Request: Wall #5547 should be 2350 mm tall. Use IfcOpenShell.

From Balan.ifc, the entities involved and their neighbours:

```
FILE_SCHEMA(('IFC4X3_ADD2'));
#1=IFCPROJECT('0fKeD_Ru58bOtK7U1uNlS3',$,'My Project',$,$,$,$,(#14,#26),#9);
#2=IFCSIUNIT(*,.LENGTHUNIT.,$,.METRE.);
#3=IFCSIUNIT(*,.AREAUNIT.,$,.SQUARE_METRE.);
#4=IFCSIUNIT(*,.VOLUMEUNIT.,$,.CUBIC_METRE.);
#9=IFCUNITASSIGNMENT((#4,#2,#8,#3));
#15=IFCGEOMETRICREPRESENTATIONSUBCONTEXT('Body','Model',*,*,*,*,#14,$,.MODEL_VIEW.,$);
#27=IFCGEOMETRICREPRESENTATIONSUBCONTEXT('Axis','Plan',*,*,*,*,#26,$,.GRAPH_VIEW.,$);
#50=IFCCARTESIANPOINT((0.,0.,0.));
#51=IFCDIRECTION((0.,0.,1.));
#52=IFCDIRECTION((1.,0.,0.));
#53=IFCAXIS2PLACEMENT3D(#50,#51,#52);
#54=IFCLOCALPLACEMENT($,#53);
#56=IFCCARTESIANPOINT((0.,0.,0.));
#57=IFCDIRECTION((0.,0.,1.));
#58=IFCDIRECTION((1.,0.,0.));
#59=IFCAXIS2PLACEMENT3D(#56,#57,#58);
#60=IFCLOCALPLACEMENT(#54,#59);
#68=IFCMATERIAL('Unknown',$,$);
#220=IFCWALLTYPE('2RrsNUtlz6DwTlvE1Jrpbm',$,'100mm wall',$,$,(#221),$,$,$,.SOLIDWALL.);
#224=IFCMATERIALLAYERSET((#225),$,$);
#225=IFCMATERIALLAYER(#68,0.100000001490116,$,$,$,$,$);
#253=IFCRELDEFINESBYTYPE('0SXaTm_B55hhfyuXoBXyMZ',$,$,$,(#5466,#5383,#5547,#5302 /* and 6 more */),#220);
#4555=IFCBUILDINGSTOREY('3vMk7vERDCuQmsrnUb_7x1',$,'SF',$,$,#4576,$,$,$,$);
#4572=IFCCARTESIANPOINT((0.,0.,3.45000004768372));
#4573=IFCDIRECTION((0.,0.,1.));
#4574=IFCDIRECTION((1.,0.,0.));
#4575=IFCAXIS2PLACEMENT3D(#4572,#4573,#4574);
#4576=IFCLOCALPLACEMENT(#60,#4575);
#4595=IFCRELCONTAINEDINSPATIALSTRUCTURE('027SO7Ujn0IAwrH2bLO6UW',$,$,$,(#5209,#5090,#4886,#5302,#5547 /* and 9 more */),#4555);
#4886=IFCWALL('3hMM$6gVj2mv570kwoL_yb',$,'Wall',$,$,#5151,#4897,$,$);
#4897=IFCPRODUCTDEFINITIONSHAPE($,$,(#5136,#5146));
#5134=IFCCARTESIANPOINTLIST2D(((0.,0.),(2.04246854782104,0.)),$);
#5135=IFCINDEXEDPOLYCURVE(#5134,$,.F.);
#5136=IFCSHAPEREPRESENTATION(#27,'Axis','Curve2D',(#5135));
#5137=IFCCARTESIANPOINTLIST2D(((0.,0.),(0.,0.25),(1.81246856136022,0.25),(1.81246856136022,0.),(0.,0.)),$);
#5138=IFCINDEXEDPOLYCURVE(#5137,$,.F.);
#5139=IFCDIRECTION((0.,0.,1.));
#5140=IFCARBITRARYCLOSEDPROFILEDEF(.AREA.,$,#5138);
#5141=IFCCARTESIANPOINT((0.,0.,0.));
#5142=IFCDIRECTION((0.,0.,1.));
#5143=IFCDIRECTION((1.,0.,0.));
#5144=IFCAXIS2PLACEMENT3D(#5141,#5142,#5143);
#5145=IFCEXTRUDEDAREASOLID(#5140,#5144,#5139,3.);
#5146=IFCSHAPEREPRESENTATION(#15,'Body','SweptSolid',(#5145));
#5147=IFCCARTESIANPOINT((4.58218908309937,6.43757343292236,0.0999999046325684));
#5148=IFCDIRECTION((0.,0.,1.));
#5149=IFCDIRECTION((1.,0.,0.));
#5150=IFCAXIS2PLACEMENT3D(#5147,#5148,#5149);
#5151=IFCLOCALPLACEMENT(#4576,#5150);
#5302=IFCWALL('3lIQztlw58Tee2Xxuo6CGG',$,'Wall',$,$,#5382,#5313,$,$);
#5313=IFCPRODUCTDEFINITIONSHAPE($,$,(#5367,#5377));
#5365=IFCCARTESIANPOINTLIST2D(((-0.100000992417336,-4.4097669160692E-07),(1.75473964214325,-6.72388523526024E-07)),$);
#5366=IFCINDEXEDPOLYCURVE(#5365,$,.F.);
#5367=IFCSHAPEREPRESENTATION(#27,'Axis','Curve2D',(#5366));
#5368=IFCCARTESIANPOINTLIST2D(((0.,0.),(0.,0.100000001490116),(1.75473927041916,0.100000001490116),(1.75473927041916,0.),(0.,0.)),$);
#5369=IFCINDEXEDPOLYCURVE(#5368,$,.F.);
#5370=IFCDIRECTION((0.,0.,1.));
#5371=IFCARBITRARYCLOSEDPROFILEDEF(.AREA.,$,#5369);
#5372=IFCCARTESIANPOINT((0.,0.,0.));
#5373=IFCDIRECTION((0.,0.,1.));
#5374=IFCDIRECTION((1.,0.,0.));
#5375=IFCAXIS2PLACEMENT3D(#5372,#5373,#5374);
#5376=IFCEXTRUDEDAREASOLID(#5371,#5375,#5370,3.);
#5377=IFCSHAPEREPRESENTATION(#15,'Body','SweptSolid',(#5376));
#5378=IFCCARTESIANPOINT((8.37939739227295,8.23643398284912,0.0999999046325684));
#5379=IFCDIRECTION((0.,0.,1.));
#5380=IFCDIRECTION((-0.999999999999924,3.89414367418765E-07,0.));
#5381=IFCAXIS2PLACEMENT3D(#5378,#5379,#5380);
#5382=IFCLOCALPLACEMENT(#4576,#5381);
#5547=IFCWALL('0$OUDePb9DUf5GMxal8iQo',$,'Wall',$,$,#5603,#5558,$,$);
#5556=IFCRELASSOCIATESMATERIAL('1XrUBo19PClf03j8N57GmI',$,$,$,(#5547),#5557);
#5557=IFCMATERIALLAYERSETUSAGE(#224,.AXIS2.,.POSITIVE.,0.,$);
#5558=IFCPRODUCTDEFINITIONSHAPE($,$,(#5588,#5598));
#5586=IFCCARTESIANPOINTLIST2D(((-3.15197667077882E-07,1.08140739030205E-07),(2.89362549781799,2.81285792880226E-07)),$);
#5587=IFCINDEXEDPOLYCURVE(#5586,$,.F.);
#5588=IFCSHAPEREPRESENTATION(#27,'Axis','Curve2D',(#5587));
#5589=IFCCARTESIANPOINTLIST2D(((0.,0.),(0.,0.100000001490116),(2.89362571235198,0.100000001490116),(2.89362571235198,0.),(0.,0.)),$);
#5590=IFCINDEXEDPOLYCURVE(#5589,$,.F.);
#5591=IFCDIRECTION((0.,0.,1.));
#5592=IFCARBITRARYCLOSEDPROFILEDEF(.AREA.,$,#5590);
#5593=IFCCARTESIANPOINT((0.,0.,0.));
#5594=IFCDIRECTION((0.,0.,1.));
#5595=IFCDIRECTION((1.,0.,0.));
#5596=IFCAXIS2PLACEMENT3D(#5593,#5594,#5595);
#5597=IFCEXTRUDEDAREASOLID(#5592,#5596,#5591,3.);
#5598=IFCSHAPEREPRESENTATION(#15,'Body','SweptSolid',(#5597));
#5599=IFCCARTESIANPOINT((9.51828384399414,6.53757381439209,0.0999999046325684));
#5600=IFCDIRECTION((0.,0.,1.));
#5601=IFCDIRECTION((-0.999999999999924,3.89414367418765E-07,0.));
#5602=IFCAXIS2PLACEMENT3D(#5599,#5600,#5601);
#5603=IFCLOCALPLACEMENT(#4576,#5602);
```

```python
import ifcopenshell
import ifcopenshell.geom
import ifcopenshell.util.representation
import ifcopenshell.util.shape
import ifcopenshell.util.unit

model = ifcopenshell.open("Balan.ifc")
unit_scale = ifcopenshell.util.unit.calculate_unit_scale(model)
settings = ifcopenshell.geom.settings()


def volume(element):
    """Net volume in cubic metres, openings subtracted."""
    shape = ifcopenshell.geom.create_shape(settings, element)
    return ifcopenshell.util.shape.get_volume(shape.geometry)


wall = model.by_guid("0$OUDePb9DUf5GMxal8iQo")
before = volume(wall)

body = ifcopenshell.util.representation.get_representation(wall, "Model", "Body")
solid = body.Items[0]
old_height = solid.Depth
solid.Depth = 2.35 / unit_scale
after = volume(wall)

print(f"height {old_height:g} -> {solid.Depth:g}, volume {before:.3f} -> {after:.3f} m3")

model.write("Balan_edited.ifc")
```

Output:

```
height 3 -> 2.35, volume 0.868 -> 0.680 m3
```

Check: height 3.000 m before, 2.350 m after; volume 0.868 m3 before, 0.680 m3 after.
